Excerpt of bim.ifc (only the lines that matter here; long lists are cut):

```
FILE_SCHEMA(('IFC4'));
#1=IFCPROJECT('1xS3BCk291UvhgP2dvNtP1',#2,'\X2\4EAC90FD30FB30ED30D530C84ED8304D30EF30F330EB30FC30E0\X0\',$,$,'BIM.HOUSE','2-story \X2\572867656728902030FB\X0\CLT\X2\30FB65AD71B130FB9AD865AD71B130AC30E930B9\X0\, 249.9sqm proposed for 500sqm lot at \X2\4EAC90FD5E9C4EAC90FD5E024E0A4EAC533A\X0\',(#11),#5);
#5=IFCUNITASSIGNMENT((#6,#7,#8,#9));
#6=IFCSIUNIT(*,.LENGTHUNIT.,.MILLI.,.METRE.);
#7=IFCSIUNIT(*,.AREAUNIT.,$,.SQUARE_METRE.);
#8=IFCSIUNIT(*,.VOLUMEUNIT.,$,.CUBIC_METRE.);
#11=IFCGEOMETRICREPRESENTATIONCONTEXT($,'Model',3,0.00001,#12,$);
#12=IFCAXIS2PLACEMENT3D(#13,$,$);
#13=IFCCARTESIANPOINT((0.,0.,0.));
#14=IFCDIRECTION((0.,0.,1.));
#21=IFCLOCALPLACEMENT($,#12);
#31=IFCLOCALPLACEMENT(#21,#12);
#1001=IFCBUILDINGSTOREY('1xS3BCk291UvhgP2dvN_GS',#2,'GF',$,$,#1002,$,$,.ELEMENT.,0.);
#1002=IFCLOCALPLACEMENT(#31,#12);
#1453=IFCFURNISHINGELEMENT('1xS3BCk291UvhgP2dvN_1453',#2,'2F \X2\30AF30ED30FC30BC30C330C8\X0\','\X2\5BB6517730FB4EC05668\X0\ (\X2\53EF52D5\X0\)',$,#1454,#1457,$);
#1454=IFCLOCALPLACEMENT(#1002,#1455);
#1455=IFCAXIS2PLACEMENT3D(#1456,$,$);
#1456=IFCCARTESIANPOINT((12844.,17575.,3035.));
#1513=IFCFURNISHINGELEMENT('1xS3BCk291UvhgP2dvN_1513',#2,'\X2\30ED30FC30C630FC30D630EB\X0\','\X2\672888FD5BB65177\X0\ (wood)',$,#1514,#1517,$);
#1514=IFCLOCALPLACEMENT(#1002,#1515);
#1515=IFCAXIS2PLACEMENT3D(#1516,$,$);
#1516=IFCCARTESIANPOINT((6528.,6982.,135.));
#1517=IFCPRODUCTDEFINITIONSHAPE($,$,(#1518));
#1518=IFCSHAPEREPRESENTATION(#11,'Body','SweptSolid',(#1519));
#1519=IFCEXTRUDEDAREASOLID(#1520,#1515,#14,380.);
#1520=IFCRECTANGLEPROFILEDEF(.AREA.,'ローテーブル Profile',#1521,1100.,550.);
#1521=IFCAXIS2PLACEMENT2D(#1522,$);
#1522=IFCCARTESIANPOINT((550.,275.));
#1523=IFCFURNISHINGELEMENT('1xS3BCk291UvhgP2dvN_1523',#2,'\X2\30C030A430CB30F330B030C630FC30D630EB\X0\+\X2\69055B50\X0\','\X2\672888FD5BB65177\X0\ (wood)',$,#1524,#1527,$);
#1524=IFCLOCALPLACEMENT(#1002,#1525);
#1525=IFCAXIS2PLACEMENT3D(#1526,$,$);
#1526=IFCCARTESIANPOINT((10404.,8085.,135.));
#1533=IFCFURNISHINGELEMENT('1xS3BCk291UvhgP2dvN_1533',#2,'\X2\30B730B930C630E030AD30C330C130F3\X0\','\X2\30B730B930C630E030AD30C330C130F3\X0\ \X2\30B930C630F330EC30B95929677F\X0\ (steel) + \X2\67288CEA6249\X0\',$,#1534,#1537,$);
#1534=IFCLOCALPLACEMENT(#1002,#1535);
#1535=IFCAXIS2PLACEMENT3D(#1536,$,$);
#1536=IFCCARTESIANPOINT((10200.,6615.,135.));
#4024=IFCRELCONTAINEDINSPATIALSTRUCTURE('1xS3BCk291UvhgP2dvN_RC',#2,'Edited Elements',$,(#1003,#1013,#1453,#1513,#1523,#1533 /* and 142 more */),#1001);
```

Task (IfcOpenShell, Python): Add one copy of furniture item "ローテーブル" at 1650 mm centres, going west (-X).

```python
import numpy as np
import ifcopenshell
import ifcopenshell.api.geometry
import ifcopenshell.api.root
import ifcopenshell.util.element
import ifcopenshell.util.placement
import ifcopenshell.util.unit

model = ifcopenshell.open("bim.ifc")
unit_scale = ifcopenshell.util.unit.calculate_unit_scale(model)


def reuse_history(source, copy):
    """copy_class also copies each property set's owner history, people and application; keep the originals."""
    for rel in copy.IsDefinedBy:
        if rel.is_a("IfcRelDefinesByProperties") and (history := rel.RelatingPropertyDefinition.OwnerHistory):
            rel.RelatingPropertyDefinition.OwnerHistory = source.OwnerHistory
            ifcopenshell.util.element.remove_deep2(model, history)


source = model.by_guid("1xS3BCk291UvhgP2dvN_1513")
base = ifcopenshell.util.placement.get_local_placement(source.ObjectPlacement)
step = np.array([-1.0, 0.0, 0.0]) * 1.65 / unit_scale

for i in range(1, 2):
    copy = ifcopenshell.api.root.copy_class(model, product=source)
    copy.Representation = ifcopenshell.util.element.copy_deep(
        model, source.Representation, exclude=["IfcGeometricRepresentationContext", "IfcRepresentationMap"]
    )
    reuse_history(source, copy)
    matrix = base.copy()
    matrix[:3, 3] += i * step
    print("added at", matrix[:3, 3].round(3) + 0.0)
    ifcopenshell.api.geometry.edit_object_placement(model, product=copy, matrix=matrix, is_si=False)

model.write("bim_rev.ifc")
```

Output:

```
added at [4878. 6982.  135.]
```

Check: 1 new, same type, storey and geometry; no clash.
